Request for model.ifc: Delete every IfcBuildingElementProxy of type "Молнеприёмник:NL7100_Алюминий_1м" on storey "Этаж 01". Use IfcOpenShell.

First a look at what the model holds.

```python
import ifcopenshell
import ifcopenshell.util.element

model = ifcopenshell.open("model.ifc")
print(model.schema)
storey = next(s for s in model.by_type("IfcBuildingStorey") if s.Name == "Этаж 01")
proxies = [e for e in ifcopenshell.util.element.get_decomposition(storey) if e.is_a("IfcBuildingElementProxy")]
seen = {}
for e in proxies:
    element_type = ifcopenshell.util.element.get_type(e)
    name = element_type.Name if element_type not in (None, e) else None
    seen[name] = seen.get(name, 0) + 1
for name, count in sorted(seen.items(), key=str):
    print(count, "x", name)
```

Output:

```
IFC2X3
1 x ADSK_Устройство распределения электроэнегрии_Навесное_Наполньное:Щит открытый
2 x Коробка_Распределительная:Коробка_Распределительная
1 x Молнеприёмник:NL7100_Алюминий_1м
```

```python
import ifcopenshell
import ifcopenshell.api.root
import ifcopenshell.util.element

model = ifcopenshell.open("model.ifc")

storey = next(s for s in model.by_type("IfcBuildingStorey") if s.Name == "Этаж 01")
proxies = [e for e in ifcopenshell.util.element.get_decomposition(storey) if e.is_a("IfcBuildingElementProxy")]
targets = [e for e in proxies if (t := ifcopenshell.util.element.get_type(e)) not in (None, e) and t.Name == "Молнеприёмник:NL7100_Алюминий_1м"]

for e in targets:
    ifcopenshell.api.root.remove_product(model, product=e)
print(len(targets), "removed")

model.write("model_rev.ifc")
```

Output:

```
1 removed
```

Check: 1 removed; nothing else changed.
